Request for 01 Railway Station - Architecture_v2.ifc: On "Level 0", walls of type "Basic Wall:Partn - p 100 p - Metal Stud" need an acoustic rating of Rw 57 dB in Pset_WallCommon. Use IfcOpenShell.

First a look at what the model holds.

```python
import ifcopenshell
import ifcopenshell.util.element

model = ifcopenshell.open("01 Railway Station - Architecture_v2.ifc")
print(model.schema)
storey = next(s for s in model.by_type("IfcBuildingStorey") if s.Name == "Level 0")
walls = [e for e in ifcopenshell.util.element.get_decomposition(storey) if e.is_a("IfcWall")]
seen = {}
for e in walls:
    element_type = ifcopenshell.util.element.get_type(e)
    key = (element_type.Name if element_type != e and element_type else None, ifcopenshell.util.element.get_pset(e, "Pset_WallCommon", "AcousticRating"))
    seen[key] = seen.get(key, 0) + 1
for (name, value), count in sorted(seen.items(), key=str):
    print(count, "x", name, "|", value)
```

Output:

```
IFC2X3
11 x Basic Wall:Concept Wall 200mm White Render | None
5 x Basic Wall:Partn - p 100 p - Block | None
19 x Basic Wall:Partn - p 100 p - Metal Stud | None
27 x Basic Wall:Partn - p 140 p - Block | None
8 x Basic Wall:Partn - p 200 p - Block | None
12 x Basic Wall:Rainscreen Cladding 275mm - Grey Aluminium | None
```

```python
import ifcopenshell
import ifcopenshell.api.pset
import ifcopenshell.util.element

model = ifcopenshell.open("01 Railway Station - Architecture_v2.ifc")

storey = next(s for s in model.by_type("IfcBuildingStorey") if s.Name == "Level 0")
walls = [e for e in ifcopenshell.util.element.get_decomposition(storey) if e.is_a("IfcWall")]

count = 0
for e in walls:
    element_type = ifcopenshell.util.element.get_type(e)
    if element_type in (None, e) or element_type.Name != "Basic Wall:Partn - p 100 p - Metal Stud":
        continue
    # add_pset returns the element's existing set when there is one.
    pset = ifcopenshell.api.pset.add_pset(model, product=e, name="Pset_WallCommon")
    ifcopenshell.api.pset.edit_pset(model, pset=pset, properties={"AcousticRating": "Rw 57 dB"})
    count += 1

print(count, "walls updated")

model.write("01 Railway Station - Architecture_v2_rev.ifc")
```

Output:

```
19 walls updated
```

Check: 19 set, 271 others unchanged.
